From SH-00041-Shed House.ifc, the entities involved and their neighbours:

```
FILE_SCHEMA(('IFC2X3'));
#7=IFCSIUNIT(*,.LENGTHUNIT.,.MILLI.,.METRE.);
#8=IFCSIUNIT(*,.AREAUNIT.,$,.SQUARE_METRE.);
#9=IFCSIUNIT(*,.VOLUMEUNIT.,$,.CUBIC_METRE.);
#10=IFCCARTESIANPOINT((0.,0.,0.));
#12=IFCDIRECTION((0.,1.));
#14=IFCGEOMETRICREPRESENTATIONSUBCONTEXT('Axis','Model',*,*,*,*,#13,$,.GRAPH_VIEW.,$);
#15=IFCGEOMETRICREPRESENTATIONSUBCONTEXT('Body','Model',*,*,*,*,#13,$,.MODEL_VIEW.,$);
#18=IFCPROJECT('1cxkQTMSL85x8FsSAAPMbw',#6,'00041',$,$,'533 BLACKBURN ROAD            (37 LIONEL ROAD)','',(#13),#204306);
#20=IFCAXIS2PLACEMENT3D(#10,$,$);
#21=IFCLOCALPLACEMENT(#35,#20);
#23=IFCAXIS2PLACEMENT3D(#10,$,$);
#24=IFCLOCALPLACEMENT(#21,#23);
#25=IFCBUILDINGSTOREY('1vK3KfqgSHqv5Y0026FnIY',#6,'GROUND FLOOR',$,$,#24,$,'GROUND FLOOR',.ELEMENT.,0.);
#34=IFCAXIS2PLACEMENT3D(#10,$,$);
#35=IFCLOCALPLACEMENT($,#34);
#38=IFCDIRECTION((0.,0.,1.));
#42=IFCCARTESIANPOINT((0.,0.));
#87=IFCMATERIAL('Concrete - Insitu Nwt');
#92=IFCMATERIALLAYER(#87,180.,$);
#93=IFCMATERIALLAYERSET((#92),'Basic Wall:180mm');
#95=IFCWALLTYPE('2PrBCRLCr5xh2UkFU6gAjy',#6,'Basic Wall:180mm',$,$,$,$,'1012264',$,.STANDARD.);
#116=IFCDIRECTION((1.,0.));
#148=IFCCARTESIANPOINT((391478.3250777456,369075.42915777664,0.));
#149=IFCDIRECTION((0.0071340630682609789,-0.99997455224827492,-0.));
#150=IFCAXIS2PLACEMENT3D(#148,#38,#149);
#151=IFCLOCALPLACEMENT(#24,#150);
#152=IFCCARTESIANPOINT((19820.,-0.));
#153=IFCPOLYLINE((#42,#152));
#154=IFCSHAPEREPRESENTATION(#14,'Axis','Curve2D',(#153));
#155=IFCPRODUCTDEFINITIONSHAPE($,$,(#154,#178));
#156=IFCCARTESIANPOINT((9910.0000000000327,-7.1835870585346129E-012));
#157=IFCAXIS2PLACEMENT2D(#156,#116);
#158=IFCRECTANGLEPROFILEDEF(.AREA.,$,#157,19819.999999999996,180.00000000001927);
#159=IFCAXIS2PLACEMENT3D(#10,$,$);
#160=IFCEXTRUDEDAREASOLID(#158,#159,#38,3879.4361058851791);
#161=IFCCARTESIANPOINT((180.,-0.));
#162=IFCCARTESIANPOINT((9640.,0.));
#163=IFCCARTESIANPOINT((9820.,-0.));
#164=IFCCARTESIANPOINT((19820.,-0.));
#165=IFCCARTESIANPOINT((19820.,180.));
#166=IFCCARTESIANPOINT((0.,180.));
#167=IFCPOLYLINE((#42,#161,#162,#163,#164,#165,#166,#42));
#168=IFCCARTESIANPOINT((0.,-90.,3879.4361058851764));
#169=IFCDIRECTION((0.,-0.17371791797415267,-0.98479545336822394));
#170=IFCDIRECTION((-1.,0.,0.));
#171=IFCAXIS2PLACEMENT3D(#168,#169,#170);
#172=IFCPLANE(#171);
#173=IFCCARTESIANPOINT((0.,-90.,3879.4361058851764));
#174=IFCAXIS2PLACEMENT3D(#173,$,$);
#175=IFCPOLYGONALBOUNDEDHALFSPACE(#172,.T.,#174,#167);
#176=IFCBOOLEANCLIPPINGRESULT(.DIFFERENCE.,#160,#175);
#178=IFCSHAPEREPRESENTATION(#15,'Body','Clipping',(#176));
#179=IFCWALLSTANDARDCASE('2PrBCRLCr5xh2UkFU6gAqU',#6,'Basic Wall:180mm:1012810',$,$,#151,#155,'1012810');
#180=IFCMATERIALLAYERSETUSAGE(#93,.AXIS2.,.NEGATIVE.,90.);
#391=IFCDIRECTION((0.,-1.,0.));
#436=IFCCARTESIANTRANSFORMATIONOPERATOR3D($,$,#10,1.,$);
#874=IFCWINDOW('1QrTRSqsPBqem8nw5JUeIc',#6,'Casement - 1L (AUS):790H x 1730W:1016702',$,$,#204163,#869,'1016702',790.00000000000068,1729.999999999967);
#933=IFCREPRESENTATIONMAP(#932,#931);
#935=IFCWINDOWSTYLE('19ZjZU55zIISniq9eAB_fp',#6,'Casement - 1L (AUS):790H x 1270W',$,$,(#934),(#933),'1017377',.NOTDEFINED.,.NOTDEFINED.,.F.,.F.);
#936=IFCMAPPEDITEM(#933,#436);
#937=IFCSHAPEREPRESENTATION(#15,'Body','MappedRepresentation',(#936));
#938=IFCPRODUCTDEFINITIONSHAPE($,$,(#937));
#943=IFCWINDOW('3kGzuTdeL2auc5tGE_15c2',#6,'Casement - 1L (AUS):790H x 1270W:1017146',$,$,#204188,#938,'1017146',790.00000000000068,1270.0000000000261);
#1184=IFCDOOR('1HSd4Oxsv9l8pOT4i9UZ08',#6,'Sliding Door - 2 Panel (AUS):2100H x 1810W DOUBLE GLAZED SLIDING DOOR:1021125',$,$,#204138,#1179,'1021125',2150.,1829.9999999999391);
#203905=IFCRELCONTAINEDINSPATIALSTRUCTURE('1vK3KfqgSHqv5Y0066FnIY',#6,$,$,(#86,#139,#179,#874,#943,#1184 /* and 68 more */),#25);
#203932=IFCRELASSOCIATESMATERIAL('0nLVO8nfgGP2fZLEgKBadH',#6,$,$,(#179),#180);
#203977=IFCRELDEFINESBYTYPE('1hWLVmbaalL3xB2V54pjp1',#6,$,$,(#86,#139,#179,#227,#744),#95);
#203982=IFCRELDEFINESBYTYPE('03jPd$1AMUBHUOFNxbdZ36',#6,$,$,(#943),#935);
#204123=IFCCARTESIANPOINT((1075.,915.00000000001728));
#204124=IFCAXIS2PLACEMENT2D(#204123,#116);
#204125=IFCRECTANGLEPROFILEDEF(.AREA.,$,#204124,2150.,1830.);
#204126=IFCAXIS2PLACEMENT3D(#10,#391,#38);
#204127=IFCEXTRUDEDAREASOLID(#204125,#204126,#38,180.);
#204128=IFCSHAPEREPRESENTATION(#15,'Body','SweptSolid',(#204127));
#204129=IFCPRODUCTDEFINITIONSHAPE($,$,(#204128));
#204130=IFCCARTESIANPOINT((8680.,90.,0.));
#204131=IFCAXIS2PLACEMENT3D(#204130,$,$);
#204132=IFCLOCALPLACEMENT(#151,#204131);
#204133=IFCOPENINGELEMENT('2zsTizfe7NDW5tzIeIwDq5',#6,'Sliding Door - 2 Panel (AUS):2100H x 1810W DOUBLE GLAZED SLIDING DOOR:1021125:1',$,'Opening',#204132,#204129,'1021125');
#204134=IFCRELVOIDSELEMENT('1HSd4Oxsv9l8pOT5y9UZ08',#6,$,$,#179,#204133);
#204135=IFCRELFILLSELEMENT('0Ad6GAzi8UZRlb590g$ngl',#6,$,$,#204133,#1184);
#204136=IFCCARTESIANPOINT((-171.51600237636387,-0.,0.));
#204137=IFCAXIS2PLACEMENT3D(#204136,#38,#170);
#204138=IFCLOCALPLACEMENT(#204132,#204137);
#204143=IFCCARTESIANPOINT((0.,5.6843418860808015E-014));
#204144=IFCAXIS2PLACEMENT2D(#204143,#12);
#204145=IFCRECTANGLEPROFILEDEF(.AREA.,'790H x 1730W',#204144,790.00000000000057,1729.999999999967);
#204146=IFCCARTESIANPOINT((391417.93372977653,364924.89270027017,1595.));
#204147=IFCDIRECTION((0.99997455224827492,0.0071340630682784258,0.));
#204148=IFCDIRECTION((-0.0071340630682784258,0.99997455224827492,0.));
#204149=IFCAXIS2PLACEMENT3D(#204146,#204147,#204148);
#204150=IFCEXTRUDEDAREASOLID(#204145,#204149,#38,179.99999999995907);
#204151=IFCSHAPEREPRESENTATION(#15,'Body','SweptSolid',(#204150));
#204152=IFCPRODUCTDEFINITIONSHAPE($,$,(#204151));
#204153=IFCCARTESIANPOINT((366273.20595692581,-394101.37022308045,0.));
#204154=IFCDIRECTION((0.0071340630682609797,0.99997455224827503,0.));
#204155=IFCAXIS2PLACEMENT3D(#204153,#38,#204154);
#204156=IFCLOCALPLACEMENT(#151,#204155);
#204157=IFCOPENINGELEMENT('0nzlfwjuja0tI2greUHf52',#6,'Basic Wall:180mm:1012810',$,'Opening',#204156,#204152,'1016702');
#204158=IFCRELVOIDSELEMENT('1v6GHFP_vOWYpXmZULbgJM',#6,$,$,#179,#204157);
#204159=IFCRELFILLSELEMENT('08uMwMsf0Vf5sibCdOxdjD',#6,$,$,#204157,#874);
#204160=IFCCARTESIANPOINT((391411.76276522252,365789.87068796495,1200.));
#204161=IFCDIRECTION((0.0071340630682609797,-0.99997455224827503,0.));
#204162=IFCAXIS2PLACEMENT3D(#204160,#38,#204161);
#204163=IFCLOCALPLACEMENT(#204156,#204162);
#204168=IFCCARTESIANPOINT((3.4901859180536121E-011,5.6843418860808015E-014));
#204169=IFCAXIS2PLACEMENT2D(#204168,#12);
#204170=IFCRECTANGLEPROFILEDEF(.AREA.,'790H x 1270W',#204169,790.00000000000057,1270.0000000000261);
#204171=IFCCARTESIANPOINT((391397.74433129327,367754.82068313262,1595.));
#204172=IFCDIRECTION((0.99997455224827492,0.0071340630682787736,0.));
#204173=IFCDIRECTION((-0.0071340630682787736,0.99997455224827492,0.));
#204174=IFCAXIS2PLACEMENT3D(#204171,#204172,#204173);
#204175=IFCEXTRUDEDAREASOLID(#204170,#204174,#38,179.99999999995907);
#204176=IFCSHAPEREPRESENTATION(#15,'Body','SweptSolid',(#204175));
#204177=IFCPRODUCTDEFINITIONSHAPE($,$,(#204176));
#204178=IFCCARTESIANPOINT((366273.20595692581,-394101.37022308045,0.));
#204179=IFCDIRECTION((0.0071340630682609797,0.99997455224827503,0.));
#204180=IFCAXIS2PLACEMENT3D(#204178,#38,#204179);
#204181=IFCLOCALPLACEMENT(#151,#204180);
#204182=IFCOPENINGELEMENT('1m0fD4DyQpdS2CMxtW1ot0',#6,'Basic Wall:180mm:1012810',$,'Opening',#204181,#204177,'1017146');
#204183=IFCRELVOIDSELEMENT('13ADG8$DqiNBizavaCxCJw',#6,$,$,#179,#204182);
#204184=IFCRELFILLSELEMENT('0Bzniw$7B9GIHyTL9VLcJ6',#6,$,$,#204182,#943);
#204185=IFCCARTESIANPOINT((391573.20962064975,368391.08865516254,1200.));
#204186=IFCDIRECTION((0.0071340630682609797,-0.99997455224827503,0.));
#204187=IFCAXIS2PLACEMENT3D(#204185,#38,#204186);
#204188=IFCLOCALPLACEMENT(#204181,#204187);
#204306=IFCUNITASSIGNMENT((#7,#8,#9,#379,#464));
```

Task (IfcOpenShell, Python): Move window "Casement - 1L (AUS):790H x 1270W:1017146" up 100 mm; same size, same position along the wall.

```python
import numpy as np
import ifcopenshell
import ifcopenshell.api.geometry
import ifcopenshell.util.placement
import ifcopenshell.util.unit

model = ifcopenshell.open("SH-00041-Shed House.ifc")
unit_scale = ifcopenshell.util.unit.calculate_unit_scale(model)

window = model.by_guid("3kGzuTdeL2auc5tGE_15c2")
opening = window.FillsVoids[0].RelatingOpeningElement
dz = 0.1 / unit_scale

shift = np.array([0.0, 0.0, dz])
# The window is placed relative to its opening, so it follows when the opening moves.
matrix = ifcopenshell.util.placement.get_local_placement(opening.ObjectPlacement)
matrix[:3, 3] += shift
ifcopenshell.api.geometry.edit_object_placement(
    model, product=opening, matrix=matrix, is_si=False, should_transform_children=True
)

print(f"moved by {dz * unit_scale:+.3f} m")

model.write("SH-00041-Shed House-out.ifc")
```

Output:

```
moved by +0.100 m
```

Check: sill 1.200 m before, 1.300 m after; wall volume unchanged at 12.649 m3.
